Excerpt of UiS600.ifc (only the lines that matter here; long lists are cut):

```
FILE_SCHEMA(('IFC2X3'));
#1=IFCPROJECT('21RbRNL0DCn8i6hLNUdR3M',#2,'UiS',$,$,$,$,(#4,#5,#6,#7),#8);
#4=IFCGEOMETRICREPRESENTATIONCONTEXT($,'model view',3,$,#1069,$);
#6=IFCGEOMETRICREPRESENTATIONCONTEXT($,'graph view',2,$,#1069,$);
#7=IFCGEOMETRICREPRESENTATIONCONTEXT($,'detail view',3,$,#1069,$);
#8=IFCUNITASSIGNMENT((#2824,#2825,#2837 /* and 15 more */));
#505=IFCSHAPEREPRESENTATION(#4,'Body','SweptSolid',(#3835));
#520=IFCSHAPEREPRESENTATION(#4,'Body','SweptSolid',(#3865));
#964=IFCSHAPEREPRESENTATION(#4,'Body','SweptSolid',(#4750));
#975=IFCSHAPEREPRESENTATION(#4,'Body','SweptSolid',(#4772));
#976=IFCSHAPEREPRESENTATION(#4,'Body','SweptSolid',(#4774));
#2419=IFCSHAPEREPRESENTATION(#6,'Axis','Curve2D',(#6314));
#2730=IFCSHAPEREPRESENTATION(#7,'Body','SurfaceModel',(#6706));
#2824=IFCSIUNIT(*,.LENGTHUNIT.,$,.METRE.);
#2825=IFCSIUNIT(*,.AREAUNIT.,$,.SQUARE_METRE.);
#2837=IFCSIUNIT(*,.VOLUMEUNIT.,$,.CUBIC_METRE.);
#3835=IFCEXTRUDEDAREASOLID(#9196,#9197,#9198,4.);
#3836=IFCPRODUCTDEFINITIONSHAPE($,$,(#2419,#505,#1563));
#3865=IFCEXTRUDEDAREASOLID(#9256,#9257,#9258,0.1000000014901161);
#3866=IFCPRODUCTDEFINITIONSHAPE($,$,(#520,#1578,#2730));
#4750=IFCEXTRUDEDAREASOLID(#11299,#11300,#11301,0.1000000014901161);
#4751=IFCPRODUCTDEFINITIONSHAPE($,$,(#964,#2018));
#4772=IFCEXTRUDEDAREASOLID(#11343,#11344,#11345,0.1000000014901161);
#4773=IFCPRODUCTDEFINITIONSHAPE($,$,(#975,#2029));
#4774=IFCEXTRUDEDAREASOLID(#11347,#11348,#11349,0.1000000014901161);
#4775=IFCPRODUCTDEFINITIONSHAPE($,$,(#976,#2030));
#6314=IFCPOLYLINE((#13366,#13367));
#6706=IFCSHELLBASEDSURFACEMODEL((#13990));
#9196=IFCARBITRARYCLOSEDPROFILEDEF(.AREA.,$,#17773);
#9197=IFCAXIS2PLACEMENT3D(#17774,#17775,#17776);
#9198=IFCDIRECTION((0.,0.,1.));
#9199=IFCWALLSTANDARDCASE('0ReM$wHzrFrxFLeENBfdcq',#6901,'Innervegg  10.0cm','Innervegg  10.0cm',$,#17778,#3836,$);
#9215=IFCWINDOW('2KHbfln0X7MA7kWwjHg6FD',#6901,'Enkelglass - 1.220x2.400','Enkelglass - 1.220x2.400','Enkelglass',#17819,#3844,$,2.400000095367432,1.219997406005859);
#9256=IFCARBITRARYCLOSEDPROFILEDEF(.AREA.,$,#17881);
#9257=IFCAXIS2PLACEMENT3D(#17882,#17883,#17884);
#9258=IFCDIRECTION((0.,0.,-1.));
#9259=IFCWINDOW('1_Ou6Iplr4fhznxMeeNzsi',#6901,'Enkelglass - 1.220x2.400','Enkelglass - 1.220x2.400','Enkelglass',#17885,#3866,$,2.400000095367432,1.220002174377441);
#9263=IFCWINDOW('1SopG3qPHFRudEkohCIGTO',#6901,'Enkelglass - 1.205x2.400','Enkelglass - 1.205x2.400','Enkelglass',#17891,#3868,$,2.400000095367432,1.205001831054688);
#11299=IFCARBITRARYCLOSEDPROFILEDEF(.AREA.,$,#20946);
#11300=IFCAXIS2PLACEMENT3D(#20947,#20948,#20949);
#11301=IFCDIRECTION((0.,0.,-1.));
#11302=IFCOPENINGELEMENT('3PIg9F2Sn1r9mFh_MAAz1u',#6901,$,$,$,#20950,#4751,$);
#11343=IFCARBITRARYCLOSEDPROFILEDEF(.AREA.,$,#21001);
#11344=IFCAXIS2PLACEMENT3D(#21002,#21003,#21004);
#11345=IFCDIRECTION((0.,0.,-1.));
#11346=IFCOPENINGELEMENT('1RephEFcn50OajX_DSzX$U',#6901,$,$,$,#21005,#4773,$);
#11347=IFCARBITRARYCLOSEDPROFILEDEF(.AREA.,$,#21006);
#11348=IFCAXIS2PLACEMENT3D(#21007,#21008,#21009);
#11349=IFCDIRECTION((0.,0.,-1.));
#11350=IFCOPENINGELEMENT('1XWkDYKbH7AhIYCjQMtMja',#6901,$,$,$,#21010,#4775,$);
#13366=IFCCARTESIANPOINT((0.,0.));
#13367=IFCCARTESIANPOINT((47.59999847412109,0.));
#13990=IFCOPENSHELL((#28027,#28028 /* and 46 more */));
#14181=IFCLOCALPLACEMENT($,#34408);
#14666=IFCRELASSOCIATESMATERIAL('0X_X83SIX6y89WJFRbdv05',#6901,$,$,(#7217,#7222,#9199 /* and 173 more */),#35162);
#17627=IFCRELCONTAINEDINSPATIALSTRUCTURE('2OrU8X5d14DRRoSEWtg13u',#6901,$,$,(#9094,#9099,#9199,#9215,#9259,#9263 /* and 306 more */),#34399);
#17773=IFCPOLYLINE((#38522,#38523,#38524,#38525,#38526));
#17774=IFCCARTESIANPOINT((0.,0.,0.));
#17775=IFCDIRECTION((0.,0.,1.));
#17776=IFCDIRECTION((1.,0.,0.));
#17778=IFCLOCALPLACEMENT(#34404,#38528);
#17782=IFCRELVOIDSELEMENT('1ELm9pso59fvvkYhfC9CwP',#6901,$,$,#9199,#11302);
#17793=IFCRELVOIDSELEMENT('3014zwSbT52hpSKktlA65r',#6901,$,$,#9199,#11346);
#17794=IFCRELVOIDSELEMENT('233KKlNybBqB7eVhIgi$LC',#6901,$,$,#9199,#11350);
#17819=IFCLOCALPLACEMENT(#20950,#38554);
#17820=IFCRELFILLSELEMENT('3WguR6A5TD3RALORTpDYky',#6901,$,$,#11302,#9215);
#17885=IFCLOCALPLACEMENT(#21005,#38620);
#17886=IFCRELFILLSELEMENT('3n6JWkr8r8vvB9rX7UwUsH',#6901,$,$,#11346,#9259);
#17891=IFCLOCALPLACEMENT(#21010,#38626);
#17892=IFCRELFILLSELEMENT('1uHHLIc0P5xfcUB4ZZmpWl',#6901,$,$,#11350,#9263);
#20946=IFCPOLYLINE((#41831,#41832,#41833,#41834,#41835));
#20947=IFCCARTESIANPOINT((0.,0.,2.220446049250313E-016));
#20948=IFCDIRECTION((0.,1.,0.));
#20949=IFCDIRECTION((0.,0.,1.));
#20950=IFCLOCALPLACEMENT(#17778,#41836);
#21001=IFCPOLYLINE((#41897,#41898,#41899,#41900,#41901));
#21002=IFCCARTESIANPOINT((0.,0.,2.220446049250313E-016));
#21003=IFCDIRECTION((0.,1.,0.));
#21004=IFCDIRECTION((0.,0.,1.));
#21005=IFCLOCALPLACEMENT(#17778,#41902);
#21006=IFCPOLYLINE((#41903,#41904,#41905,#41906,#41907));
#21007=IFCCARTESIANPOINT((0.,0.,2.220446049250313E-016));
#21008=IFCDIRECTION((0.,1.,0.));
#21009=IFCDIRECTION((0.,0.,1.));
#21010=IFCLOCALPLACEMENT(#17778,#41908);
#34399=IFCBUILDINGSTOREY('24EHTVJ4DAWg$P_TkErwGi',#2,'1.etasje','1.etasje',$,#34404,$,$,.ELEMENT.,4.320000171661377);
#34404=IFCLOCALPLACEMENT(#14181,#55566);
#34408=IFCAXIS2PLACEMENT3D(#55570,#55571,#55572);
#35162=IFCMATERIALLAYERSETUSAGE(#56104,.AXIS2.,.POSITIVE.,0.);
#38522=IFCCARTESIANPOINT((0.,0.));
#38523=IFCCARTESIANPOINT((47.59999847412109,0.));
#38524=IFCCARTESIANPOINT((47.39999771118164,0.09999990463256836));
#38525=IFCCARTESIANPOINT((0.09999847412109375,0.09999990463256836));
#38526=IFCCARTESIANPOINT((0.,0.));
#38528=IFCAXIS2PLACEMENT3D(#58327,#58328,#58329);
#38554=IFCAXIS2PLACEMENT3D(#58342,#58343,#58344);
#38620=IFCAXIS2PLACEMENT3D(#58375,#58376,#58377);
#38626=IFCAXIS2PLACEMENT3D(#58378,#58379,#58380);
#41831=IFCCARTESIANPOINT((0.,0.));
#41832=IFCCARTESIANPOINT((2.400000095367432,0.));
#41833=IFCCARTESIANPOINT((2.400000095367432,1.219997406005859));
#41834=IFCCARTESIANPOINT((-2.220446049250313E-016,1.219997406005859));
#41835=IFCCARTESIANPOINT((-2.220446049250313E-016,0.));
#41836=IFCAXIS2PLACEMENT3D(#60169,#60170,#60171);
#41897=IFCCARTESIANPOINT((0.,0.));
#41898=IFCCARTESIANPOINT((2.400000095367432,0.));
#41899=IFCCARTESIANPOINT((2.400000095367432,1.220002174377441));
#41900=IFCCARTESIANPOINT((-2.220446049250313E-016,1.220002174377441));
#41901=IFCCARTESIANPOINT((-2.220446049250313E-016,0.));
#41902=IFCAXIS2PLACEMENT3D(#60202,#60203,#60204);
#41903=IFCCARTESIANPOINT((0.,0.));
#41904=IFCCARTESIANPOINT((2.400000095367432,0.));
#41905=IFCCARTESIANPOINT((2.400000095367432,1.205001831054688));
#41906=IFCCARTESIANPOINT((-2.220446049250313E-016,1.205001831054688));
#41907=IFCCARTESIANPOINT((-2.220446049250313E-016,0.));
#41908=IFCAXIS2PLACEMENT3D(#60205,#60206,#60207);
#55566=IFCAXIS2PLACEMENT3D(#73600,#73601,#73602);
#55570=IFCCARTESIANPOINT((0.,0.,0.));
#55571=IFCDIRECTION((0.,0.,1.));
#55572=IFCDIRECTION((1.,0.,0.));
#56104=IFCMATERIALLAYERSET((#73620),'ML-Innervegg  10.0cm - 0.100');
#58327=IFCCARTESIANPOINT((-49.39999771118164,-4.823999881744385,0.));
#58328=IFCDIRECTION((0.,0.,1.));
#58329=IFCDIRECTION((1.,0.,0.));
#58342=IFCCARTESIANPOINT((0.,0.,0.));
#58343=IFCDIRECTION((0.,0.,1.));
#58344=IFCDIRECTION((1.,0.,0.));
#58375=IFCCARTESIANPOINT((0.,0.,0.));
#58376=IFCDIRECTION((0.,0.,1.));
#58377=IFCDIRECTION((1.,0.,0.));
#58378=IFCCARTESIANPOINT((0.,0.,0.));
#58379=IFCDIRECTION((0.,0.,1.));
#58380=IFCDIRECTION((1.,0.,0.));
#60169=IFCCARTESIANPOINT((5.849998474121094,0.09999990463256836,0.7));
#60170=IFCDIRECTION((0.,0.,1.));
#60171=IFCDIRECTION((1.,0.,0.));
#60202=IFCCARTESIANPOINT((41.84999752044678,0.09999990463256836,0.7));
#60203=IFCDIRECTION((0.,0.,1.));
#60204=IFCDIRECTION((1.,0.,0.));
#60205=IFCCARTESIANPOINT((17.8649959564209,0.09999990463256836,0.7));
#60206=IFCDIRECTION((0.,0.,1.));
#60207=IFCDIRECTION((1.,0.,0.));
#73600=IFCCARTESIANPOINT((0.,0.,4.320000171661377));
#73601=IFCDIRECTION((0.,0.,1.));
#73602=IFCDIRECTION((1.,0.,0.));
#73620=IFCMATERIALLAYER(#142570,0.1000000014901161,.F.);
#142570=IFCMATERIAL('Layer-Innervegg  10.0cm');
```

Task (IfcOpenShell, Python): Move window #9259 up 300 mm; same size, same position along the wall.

```python
import numpy as np
import ifcopenshell
import ifcopenshell.api.geometry
import ifcopenshell.util.placement
import ifcopenshell.util.unit

model = ifcopenshell.open("UiS600.ifc")
unit_scale = ifcopenshell.util.unit.calculate_unit_scale(model)

window = model.by_guid("1_Ou6Iplr4fhznxMeeNzsi")
opening = window.FillsVoids[0].RelatingOpeningElement
dz = 0.3 / unit_scale

shift = np.array([0.0, 0.0, dz])
# The window is placed relative to its opening, so it follows when the opening moves.
matrix = ifcopenshell.util.placement.get_local_placement(opening.ObjectPlacement)
matrix[:3, 3] += shift
ifcopenshell.api.geometry.edit_object_placement(
    model, product=opening, matrix=matrix, is_si=False, should_transform_children=True
)

print(f"moved by {dz * unit_scale:+.3f} m")

model.write("UiS600-out.ifc")
```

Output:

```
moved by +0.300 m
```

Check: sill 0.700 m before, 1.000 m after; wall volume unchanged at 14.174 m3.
